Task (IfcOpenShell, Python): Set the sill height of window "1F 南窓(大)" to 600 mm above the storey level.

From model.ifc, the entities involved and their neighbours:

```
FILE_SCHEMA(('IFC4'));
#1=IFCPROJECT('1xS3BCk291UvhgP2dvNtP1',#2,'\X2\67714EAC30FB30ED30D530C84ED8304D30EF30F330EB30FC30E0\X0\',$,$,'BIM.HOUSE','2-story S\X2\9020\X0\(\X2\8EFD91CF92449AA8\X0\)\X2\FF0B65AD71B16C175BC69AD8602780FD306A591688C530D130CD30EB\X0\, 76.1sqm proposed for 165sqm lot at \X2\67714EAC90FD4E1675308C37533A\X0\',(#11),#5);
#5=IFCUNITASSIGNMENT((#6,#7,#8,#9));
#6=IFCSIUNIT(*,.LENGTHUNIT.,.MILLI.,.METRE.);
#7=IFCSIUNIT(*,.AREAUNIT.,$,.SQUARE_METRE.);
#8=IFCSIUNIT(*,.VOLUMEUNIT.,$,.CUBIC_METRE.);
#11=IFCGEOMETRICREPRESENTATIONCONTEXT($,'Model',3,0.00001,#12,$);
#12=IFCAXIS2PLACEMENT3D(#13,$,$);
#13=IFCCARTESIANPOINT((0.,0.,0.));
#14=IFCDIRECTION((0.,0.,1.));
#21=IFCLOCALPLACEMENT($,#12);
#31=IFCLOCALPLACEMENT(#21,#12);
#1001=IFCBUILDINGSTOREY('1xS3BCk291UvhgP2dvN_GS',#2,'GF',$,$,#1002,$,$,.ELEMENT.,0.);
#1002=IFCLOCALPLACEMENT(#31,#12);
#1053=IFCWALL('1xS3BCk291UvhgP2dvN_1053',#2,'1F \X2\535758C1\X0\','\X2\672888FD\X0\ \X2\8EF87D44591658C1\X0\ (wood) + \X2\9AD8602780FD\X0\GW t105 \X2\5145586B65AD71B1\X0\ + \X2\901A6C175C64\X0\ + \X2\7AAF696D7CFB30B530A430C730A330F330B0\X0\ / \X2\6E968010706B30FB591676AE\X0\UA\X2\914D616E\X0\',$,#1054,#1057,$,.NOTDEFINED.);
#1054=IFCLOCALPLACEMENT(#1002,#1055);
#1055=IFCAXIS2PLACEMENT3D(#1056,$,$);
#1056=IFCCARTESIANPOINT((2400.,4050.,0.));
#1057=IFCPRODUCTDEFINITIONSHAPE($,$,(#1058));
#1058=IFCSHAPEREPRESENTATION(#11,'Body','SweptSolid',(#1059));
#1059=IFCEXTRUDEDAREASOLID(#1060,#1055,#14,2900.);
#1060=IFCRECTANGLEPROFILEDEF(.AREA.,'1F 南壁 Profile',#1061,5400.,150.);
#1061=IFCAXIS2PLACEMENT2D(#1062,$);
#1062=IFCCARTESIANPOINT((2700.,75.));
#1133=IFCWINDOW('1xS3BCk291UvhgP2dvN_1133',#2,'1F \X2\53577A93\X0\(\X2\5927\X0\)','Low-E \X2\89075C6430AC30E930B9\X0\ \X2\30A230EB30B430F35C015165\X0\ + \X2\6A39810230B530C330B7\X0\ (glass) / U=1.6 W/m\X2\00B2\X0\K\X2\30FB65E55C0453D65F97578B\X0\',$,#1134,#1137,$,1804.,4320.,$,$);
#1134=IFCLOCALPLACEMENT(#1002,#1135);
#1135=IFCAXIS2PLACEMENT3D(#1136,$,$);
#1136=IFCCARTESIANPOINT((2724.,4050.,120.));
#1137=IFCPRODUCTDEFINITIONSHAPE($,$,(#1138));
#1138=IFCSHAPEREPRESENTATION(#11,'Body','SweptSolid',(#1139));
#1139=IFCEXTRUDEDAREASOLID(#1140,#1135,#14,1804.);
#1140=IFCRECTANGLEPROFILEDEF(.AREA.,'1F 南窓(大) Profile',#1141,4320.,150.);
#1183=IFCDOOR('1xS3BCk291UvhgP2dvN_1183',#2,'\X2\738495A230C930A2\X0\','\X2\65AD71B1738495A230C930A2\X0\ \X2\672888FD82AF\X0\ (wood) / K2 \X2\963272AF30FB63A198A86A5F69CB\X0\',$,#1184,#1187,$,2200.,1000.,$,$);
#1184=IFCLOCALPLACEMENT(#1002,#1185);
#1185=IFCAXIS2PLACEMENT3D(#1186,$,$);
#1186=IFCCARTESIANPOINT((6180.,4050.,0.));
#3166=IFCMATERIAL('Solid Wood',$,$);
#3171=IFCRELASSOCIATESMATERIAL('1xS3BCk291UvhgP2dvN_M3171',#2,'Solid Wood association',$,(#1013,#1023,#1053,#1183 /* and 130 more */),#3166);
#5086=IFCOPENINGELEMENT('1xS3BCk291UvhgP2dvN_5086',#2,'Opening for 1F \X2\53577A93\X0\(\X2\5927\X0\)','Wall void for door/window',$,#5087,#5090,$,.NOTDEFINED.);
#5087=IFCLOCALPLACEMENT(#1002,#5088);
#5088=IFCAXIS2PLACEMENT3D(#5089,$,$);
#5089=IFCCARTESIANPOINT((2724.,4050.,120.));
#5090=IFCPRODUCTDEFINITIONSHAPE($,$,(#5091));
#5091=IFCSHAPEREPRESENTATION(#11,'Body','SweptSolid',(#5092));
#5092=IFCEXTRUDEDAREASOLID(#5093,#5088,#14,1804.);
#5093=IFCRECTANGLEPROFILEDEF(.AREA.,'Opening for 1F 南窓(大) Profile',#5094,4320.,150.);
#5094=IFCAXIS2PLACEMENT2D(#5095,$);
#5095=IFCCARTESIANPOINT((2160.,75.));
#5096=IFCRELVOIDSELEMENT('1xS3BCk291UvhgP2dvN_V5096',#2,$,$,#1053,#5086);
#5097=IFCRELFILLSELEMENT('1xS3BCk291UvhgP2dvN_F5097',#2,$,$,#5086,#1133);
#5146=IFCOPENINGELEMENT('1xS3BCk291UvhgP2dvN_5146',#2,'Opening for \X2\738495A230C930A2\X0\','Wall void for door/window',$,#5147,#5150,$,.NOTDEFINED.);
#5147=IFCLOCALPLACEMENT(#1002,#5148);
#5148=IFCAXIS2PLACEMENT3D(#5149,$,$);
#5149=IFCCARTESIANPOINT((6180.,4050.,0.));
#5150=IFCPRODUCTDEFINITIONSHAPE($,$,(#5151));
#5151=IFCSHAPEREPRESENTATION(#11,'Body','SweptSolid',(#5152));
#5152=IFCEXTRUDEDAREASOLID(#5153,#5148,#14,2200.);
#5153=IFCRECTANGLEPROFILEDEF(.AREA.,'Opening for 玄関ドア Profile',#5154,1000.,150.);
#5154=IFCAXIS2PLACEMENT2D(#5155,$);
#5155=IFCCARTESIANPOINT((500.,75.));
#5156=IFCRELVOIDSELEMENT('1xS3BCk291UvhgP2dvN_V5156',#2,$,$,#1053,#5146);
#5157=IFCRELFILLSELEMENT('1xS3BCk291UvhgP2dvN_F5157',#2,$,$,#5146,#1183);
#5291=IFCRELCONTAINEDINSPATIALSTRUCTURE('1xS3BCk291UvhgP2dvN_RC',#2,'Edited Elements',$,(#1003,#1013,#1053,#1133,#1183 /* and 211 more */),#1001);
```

```python
import numpy as np
import ifcopenshell
import ifcopenshell.api.geometry
import ifcopenshell.geom
import ifcopenshell.util.element
import ifcopenshell.util.placement
import ifcopenshell.util.shape
import ifcopenshell.util.unit

model = ifcopenshell.open("model.ifc")
unit_scale = ifcopenshell.util.unit.calculate_unit_scale(model)

window = model.by_guid("1xS3BCk291UvhgP2dvN_1133")
opening = window.FillsVoids[0].RelatingOpeningElement
storey = ifcopenshell.util.element.get_container(window, ifc_class="IfcBuildingStorey")
level = ifcopenshell.util.placement.get_local_placement(storey.ObjectPlacement)[2, 3]

# The opening's origin need not be at the sill, so measure its lowest point.
shape = ifcopenshell.geom.create_shape(ifcopenshell.geom.settings(), opening)
bottom = ifcopenshell.util.shape.get_shape_bottom_elevation(shape, shape.geometry) / unit_scale
dz = level + 0.6 / unit_scale - bottom

shift = np.array([0.0, 0.0, dz])
# The window is not placed relative to its opening, so move both.
for product in (opening, window):
    matrix = ifcopenshell.util.placement.get_local_placement(product.ObjectPlacement)
    matrix[:3, 3] += shift
    ifcopenshell.api.geometry.edit_object_placement(model, product=product, matrix=matrix, is_si=False)

print(f"moved by {dz * unit_scale:+.3f} m")

model.write("model_rev.ifc")
```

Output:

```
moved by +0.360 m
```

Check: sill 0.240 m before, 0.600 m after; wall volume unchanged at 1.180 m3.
